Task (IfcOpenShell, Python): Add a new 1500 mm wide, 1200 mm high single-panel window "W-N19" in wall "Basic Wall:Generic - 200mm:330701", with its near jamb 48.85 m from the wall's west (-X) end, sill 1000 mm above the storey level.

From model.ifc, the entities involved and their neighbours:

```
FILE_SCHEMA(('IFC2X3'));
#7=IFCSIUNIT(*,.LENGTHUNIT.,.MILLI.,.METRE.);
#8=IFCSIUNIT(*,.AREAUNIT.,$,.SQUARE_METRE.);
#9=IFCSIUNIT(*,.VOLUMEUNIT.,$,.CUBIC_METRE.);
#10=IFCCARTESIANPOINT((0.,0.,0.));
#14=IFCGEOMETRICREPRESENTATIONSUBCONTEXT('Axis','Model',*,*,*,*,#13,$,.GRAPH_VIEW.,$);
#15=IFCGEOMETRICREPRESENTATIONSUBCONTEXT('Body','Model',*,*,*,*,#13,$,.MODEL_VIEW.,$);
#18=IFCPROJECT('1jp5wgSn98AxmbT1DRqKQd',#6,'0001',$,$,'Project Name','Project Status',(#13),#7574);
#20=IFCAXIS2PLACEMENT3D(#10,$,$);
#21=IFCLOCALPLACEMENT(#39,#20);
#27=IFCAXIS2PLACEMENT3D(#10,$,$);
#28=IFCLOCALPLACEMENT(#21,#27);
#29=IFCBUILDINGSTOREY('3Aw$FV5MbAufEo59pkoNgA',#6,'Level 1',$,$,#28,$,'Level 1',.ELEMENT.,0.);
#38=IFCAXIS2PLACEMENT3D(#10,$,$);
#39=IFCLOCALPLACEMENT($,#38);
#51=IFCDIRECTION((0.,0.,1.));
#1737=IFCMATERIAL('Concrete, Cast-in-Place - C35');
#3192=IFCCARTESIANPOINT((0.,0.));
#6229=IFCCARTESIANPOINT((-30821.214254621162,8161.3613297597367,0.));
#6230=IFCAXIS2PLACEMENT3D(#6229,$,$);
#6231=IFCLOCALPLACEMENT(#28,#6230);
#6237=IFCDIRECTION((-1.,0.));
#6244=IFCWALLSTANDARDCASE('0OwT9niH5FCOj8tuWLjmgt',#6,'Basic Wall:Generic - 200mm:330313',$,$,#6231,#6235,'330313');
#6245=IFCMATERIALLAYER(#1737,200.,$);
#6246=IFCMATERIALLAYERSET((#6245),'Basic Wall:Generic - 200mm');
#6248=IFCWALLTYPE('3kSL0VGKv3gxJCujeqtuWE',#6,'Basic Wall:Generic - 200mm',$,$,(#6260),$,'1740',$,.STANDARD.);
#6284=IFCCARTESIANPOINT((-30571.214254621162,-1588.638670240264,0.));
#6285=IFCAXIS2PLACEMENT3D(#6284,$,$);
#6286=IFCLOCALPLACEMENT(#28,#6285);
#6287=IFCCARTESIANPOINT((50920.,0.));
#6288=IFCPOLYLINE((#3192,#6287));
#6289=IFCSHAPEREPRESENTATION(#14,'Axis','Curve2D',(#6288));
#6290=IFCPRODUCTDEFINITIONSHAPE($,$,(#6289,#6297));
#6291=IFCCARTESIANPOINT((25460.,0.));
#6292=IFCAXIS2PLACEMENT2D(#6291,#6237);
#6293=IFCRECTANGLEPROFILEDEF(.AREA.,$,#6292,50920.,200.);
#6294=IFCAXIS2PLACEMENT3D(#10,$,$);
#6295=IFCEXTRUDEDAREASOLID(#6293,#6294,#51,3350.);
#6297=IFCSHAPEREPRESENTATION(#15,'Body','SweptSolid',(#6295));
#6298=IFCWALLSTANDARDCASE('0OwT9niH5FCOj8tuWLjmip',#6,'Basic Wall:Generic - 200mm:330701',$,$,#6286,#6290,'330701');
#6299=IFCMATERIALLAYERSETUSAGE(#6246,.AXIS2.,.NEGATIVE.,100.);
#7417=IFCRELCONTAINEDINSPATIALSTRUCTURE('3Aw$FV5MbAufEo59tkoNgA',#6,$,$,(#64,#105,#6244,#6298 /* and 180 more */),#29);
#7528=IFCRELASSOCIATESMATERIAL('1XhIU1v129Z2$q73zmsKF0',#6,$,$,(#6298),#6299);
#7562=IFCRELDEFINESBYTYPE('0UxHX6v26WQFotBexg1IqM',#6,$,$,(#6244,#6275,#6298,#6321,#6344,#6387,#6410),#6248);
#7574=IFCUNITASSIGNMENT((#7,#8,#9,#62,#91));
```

```python
import numpy as np
import ifcopenshell
import ifcopenshell.api.feature
import ifcopenshell.api.geometry
import ifcopenshell.api.root
import ifcopenshell.api.spatial
import ifcopenshell.api.type
import ifcopenshell.geom
import ifcopenshell.util.element
import ifcopenshell.util.placement
import ifcopenshell.util.representation
import ifcopenshell.util.shape
import ifcopenshell.util.unit

model = ifcopenshell.open("model.ifc")
unit_scale = ifcopenshell.util.unit.calculate_unit_scale(model)
settings = ifcopenshell.geom.settings()


def volume(element):
    """Net volume in cubic metres, openings subtracted."""
    shape = ifcopenshell.geom.create_shape(settings, element)
    return ifcopenshell.util.shape.get_volume(shape.geometry)


wall = model.by_guid("0OwT9niH5FCOj8tuWLjmip")
storey = ifcopenshell.util.element.get_container(wall, ifc_class="IfcBuildingStorey")
context = ifcopenshell.util.representation.get_context(model, "Model", "Body", "MODEL_VIEW")
before = volume(wall)

width, height, from_end, sill = 1.5, 1.2, 48.85, 1  # metres

# The wall runs along its own X axis, and the end named is its -X end.
wall_shape = ifcopenshell.geom.create_shape(settings, wall)
x, y, z = ifcopenshell.util.shape.get_vertices(wall_shape.geometry).T
start = x.min() + from_end
face, thickness = float(y.min()), float(y.max() - y.min())
wall_matrix = ifcopenshell.util.placement.get_local_placement(wall.ObjectPlacement)
level = ifcopenshell.util.placement.get_local_placement(storey.ObjectPlacement)[2, 3]


def in_wall(x, y):
    """Placement at x, y metres in the wall's axes, at sill height."""
    matrix = wall_matrix.copy()
    matrix[:, 3] = wall_matrix @ np.array([x / unit_scale, y / unit_scale, 0.0, 1.0])
    matrix[2, 3] = level + sill / unit_scale
    return matrix


# Opening: a box that overshoots both wall faces by 50 mm.
opening = ifcopenshell.api.root.create_entity(model, ifc_class="IfcOpeningElement")
box = ifcopenshell.api.geometry.add_wall_representation(
    model, context=context, length=width, height=height, thickness=thickness + 0.1
)
ifcopenshell.api.geometry.assign_representation(model, product=opening, representation=box)
ifcopenshell.api.geometry.edit_object_placement(model, product=opening, matrix=in_wall(start, face - 0.05), is_si=False)
ifcopenshell.api.feature.add_feature(model, feature=opening, element=wall)

window = ifcopenshell.api.root.create_entity(model, ifc_class="IfcWindow", name="W-N19")
window.OverallWidth, window.OverallHeight = width / unit_scale, height / unit_scale
body = ifcopenshell.api.geometry.add_window_representation(
    model,
    context=context,
    overall_width=window.OverallWidth,
    overall_height=window.OverallHeight,
    partition_type="SINGLE_PANEL",
)
ifcopenshell.api.geometry.assign_representation(model, product=window, representation=body)
ifcopenshell.api.spatial.assign_container(model, products=[window], relating_structure=storey)
fills = ifcopenshell.api.feature.add_filling(model, opening=opening, element=window)
fills.OwnerHistory = window.OwnerHistory  # required in IFC2X3

# IFC2X3 keeps the operation on the window style.
style = ifcopenshell.api.root.create_entity(model, ifc_class="IfcWindowStyle", name="W-N19")
style.OperationType, style.ConstructionType = "SINGLE_PANEL", "NOTDEFINED"
style.ParameterTakesPrecedence = style.Sizeable = False
ifcopenshell.api.type.assign_type(model, related_objects=[window], relating_type=style)

# Centre the window in the wall's thickness.
ifcopenshell.api.geometry.edit_object_placement(model, product=window, matrix=in_wall(start, face), is_si=False)
window_shape = ifcopenshell.geom.create_shape(settings, window)
depth = ifcopenshell.util.shape.get_vertices(window_shape.geometry)[:, 1]
offset = face + thickness / 2 - (depth.min() + depth.max()) / 2
ifcopenshell.api.geometry.edit_object_placement(model, product=window, matrix=in_wall(start, offset), is_si=False)

after = volume(wall)

print(f"wall volume {before:.3f} -> {after:.3f} m3")

model.write("model_updated.ifc")
```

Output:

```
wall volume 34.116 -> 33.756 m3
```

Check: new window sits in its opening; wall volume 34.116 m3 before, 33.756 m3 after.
